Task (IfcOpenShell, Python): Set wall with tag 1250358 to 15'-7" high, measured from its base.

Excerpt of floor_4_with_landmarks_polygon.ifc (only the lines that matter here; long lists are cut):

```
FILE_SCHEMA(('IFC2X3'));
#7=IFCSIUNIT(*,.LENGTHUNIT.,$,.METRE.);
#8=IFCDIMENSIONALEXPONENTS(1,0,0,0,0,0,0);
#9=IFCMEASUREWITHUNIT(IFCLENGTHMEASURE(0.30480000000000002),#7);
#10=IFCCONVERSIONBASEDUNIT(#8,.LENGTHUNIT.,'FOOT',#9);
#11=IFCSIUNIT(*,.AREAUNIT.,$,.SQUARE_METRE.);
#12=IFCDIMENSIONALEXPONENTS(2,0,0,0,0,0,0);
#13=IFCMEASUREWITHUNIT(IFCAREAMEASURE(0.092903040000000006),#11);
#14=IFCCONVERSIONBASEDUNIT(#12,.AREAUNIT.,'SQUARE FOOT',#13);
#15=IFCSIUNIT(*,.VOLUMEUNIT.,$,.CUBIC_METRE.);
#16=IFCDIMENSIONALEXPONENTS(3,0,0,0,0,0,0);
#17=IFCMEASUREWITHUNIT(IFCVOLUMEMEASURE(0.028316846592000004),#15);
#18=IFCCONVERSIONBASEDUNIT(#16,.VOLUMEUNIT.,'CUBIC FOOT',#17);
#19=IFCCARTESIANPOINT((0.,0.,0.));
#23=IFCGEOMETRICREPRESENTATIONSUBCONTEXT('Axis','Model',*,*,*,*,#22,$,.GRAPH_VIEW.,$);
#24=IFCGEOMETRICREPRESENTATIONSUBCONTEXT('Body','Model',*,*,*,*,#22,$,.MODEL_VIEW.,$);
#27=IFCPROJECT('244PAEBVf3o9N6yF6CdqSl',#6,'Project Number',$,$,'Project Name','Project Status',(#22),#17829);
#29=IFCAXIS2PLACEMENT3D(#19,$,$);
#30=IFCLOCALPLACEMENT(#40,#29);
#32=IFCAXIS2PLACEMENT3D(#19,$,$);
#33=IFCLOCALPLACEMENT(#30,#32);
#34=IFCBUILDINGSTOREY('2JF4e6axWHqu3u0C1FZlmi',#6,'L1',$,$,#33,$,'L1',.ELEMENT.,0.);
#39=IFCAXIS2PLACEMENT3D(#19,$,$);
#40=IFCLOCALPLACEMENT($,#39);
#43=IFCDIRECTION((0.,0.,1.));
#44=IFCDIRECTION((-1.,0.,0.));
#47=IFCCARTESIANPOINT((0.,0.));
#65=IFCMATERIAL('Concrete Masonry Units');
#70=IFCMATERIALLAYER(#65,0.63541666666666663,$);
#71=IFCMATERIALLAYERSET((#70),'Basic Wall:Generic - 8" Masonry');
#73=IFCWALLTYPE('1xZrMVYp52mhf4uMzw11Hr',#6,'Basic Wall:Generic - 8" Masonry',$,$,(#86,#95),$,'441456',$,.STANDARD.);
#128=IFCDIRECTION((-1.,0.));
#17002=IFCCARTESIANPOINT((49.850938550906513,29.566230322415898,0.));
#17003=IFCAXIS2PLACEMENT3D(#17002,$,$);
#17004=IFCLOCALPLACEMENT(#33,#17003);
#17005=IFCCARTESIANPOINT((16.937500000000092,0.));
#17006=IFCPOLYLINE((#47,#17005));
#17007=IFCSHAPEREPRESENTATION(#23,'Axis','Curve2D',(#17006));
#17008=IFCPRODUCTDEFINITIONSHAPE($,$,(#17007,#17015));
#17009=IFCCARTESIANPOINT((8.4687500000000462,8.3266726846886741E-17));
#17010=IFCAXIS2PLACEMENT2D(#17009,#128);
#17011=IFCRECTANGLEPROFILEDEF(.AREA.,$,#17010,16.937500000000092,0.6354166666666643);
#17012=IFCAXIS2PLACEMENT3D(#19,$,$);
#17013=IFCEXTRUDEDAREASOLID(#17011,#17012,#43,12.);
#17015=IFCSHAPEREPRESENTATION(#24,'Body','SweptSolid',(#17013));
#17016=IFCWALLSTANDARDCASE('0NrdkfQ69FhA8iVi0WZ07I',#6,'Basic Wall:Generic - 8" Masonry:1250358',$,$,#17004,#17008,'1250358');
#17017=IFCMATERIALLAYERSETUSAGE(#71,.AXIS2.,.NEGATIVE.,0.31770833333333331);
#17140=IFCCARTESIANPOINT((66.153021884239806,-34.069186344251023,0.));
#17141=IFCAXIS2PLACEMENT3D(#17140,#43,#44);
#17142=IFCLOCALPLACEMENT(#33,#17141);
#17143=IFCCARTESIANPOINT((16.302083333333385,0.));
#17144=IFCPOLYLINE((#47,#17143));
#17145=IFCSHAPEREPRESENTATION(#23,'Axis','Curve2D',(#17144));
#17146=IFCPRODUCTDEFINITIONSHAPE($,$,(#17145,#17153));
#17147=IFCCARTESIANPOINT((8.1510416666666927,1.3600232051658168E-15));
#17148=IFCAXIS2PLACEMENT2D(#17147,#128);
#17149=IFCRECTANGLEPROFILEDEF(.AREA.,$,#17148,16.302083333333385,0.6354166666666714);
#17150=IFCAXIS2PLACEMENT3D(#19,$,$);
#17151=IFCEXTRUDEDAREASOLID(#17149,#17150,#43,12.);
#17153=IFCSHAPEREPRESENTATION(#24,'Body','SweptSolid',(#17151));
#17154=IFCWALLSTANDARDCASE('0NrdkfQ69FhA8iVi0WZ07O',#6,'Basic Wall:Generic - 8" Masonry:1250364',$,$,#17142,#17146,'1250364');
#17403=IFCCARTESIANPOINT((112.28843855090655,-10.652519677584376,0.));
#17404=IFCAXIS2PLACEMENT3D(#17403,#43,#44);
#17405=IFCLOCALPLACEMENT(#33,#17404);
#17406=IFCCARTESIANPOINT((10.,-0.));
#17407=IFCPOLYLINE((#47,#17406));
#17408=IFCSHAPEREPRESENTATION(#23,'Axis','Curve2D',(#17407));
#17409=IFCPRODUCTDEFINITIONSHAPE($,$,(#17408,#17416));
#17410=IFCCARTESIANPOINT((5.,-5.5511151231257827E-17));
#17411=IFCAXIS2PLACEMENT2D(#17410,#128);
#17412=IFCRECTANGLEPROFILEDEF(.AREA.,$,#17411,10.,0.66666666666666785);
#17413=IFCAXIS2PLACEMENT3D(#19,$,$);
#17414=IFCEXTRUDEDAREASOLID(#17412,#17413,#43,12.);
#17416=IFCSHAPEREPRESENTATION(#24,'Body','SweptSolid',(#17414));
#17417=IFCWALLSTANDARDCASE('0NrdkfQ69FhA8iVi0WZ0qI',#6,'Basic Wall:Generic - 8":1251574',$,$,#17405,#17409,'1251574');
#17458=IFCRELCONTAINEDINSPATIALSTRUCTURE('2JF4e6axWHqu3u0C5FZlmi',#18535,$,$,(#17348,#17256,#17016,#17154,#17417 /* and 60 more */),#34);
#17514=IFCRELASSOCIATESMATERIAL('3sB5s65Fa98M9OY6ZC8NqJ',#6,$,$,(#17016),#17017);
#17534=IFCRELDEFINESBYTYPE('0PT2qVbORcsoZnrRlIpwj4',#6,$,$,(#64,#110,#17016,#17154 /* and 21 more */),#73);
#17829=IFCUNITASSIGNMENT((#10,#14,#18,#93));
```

```python
import ifcopenshell
import ifcopenshell.geom
import ifcopenshell.util.representation
import ifcopenshell.util.shape
import ifcopenshell.util.unit

model = ifcopenshell.open("floor_4_with_landmarks_polygon.ifc")
unit_scale = ifcopenshell.util.unit.calculate_unit_scale(model)
settings = ifcopenshell.geom.settings()


def volume(element):
    """Net volume in cubic metres, openings subtracted."""
    shape = ifcopenshell.geom.create_shape(settings, element)
    return ifcopenshell.util.shape.get_volume(shape.geometry)


wall = model.by_guid("0NrdkfQ69FhA8iVi0WZ07I")
before = volume(wall)

body = ifcopenshell.util.representation.get_representation(wall, "Model", "Body")
solid = body.Items[0]
old_height = solid.Depth
solid.Depth = 187 * 0.0254 / unit_scale
after = volume(wall)

print(f"height {old_height:g} -> {solid.Depth:g}, volume {before:.3f} -> {after:.3f} m3")

model.write("floor_4_with_landmarks_polygon_rev.ifc")
```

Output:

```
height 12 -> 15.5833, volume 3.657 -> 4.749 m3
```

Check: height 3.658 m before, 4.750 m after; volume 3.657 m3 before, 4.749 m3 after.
